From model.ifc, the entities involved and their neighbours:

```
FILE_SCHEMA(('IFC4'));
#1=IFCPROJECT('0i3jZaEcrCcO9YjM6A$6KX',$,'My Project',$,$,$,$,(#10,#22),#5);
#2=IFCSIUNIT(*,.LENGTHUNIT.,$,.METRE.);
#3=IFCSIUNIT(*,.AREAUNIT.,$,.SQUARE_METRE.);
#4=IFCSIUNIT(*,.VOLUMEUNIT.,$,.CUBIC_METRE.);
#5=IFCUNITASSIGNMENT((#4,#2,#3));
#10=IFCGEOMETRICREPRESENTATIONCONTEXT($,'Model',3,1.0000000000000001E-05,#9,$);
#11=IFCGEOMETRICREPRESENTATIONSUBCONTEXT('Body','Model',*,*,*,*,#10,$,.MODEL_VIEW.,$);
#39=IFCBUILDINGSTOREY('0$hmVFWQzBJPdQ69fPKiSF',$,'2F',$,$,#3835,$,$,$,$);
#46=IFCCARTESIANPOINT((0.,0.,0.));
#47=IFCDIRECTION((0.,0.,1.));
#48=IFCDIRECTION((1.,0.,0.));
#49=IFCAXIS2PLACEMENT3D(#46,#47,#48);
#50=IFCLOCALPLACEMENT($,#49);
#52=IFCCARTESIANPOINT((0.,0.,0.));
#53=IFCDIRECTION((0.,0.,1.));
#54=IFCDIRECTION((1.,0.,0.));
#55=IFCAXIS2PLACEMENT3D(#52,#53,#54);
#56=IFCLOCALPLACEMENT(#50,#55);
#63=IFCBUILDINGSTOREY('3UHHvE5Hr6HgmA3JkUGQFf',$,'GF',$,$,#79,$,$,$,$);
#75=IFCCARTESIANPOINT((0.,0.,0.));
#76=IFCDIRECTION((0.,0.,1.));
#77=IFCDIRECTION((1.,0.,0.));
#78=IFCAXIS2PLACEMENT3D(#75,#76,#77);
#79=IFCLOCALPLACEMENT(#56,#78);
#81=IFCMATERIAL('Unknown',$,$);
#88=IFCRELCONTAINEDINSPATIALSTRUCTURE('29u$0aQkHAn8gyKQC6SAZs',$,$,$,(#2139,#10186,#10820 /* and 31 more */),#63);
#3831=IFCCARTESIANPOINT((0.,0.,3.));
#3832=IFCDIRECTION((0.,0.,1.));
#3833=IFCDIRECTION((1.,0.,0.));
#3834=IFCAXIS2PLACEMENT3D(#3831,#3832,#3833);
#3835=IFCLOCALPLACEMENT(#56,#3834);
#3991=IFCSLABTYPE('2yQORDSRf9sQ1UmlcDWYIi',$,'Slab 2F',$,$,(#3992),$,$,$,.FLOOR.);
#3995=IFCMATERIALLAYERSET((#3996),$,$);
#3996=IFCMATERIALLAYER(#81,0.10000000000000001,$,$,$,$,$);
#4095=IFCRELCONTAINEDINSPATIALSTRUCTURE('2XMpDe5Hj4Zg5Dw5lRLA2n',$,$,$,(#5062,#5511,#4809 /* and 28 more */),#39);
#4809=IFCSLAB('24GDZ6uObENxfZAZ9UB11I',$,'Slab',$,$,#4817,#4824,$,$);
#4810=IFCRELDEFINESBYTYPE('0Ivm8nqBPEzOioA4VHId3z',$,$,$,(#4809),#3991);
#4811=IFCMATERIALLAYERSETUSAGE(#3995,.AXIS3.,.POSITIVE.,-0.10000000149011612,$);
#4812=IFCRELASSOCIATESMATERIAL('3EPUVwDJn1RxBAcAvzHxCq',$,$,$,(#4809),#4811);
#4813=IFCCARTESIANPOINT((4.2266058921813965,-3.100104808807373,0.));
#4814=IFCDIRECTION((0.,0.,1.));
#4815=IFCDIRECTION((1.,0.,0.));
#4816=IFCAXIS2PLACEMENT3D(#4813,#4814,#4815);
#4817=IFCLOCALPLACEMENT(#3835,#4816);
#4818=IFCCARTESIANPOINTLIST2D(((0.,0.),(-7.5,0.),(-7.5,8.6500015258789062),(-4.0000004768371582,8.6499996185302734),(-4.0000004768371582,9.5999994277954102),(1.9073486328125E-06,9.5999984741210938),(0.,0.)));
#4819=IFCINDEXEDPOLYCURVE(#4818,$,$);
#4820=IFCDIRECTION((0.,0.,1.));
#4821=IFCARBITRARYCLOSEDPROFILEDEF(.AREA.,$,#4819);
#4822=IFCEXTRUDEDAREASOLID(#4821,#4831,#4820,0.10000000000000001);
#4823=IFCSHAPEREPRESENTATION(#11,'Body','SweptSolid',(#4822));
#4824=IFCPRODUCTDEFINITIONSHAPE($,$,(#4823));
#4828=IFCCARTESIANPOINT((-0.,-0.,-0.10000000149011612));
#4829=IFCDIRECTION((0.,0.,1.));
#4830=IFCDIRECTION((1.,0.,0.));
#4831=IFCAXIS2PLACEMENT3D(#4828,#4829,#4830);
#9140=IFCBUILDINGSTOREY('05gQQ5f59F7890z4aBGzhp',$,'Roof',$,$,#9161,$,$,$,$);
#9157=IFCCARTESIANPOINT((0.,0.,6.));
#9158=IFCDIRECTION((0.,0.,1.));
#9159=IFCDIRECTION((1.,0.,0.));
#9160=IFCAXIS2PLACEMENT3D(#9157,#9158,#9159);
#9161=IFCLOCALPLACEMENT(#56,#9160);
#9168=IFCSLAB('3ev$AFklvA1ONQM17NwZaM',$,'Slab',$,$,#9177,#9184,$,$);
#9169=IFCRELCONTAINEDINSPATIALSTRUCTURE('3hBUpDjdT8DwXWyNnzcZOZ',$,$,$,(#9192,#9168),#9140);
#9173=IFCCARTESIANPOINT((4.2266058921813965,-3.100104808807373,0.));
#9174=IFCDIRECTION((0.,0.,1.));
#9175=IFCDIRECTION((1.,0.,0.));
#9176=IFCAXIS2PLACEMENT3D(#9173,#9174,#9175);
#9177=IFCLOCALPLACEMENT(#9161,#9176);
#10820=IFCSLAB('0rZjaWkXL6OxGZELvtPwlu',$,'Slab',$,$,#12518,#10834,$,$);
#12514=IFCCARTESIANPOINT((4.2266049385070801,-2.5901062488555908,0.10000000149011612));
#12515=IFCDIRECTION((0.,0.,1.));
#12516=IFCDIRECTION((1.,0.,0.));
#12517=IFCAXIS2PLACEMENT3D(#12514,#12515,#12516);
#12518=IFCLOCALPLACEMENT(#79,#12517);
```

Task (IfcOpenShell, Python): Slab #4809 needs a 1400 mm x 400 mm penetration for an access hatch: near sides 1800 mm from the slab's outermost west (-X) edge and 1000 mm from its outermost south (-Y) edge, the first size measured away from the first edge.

```python
import numpy as np
import ifcopenshell
import ifcopenshell.api.feature
import ifcopenshell.api.geometry
import ifcopenshell.api.root
import ifcopenshell.geom
import ifcopenshell.util.placement
import ifcopenshell.util.representation
import ifcopenshell.util.shape
import ifcopenshell.util.unit

model = ifcopenshell.open("model.ifc")
unit_scale = ifcopenshell.util.unit.calculate_unit_scale(model)
settings = ifcopenshell.geom.settings()


def volume(element):
    """Net volume in cubic metres, openings subtracted."""
    shape = ifcopenshell.geom.create_shape(settings, element)
    return ifcopenshell.util.shape.get_volume(shape.geometry)


slab = model.by_guid("24GDZ6uObENxfZAZ9UB11I")
before = volume(slab)

# Extent in the slab's own axes, in metres. The edges named are its -X and -Y sides.
slab_shape = ifcopenshell.geom.create_shape(settings, slab)
vertices = ifcopenshell.util.shape.get_vertices(slab_shape.geometry)
x_min, y_min, bottom = vertices.min(axis=0)
top = vertices[:, 2].max()

opening = ifcopenshell.api.root.create_entity(model, ifc_class="IfcOpeningElement", name="Access hatch opening", predefined_type="OPENING")
context = ifcopenshell.util.representation.get_context(model, "Model", "Body", "MODEL_VIEW")
width, depth = 1.4, 0.4
outline = [(0.0, 0.0), (width, 0.0), (width, depth), (0.0, depth), (0.0, 0.0)]
# Overshoot both faces by 50 mm so the cut is clean.
shape = ifcopenshell.api.geometry.add_slab_representation(
    model, context=context, depth=top - bottom + 0.1, polyline=outline
)
ifcopenshell.api.geometry.assign_representation(model, product=opening, representation=shape)

matrix = ifcopenshell.util.placement.get_local_placement(slab.ObjectPlacement)
matrix[:, 3] = matrix @ np.append(np.array([x_min + 1.8, y_min + 1, bottom - 0.05]) / unit_scale, 1.0)
ifcopenshell.api.geometry.edit_object_placement(model, product=opening, matrix=matrix, is_si=False)
ifcopenshell.api.feature.add_feature(model, feature=opening, element=slab)

after = volume(slab)

print(f"slab volume {before:.3f} -> {after:.3f} m3")

model.write("model_v2.ifc")
```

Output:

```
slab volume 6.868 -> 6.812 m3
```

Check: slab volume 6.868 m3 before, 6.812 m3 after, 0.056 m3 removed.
